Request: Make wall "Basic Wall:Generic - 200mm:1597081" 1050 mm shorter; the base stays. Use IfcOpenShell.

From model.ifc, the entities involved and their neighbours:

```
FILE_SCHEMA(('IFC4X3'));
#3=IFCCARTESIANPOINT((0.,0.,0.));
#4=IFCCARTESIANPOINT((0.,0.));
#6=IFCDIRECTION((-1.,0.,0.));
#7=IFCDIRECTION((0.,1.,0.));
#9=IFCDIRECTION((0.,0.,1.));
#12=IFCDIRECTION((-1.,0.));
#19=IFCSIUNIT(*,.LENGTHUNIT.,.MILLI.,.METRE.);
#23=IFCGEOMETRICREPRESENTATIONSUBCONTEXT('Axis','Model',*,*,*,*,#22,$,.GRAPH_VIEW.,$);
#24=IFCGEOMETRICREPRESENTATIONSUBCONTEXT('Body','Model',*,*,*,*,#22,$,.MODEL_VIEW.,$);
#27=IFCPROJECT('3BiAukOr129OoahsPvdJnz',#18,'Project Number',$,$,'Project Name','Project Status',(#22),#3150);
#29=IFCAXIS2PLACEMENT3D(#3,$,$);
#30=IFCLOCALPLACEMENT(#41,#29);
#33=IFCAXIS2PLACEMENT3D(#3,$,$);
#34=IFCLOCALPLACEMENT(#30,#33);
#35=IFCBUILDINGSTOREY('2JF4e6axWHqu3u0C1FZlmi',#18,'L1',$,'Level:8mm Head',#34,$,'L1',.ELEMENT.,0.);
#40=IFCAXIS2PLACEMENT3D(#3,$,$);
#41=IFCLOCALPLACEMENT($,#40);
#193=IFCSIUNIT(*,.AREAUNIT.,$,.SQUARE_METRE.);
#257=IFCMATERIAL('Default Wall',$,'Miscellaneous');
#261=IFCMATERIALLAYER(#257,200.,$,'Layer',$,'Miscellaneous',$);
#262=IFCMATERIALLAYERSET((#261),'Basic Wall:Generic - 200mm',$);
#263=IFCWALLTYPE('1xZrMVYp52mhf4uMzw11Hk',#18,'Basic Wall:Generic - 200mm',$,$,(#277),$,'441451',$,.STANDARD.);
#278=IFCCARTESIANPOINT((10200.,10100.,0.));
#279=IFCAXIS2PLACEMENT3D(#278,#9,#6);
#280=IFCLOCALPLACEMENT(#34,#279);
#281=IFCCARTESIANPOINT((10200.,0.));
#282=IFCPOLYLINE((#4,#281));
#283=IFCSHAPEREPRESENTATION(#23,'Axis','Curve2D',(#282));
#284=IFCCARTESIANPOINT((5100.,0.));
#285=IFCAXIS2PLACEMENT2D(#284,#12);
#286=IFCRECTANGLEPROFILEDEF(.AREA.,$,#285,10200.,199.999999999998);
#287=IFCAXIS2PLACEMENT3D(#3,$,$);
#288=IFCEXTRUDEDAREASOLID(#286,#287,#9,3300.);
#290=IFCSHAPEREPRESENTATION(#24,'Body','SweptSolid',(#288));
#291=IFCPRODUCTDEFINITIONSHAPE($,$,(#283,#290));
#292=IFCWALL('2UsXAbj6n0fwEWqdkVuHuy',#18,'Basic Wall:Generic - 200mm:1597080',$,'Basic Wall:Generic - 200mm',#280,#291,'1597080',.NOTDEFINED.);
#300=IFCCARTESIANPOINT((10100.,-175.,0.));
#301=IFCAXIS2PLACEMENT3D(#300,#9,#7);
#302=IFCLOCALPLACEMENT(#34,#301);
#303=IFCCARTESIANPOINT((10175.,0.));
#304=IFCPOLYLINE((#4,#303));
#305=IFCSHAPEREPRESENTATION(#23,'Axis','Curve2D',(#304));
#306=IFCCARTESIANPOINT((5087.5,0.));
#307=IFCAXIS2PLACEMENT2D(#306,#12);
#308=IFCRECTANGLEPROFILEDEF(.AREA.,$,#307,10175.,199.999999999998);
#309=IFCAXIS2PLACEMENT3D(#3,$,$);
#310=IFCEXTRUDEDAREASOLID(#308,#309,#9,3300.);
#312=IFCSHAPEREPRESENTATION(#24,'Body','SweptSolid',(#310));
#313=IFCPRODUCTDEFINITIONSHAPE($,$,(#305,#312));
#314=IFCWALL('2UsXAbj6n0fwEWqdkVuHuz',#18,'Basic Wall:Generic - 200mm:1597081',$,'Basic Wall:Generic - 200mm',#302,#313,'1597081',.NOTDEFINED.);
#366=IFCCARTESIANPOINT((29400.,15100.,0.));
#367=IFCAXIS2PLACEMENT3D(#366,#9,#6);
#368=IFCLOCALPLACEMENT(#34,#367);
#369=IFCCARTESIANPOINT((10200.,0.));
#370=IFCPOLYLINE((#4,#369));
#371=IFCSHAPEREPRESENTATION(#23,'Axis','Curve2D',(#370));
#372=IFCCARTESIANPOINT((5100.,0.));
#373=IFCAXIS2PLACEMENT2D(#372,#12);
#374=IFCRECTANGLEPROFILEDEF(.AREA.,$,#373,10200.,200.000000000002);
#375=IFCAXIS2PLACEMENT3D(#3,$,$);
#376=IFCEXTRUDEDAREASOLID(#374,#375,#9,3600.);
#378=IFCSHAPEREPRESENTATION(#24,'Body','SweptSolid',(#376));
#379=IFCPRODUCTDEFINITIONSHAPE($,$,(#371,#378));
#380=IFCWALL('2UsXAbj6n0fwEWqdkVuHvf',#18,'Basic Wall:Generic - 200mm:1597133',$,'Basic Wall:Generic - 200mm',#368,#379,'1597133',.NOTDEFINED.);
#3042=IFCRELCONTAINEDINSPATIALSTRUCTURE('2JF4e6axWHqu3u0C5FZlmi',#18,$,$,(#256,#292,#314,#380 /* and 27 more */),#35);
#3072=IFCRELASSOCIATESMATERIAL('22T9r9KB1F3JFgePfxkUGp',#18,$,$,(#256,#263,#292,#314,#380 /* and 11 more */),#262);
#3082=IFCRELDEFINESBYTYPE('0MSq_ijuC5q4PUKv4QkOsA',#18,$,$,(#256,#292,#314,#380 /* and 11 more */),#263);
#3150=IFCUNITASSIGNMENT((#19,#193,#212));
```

```python
import ifcopenshell
import ifcopenshell.geom
import ifcopenshell.util.representation
import ifcopenshell.util.shape
import ifcopenshell.util.unit

model = ifcopenshell.open("model.ifc")
unit_scale = ifcopenshell.util.unit.calculate_unit_scale(model)
settings = ifcopenshell.geom.settings()


def volume(element):
    """Net volume in cubic metres, openings subtracted."""
    shape = ifcopenshell.geom.create_shape(settings, element)
    return ifcopenshell.util.shape.get_volume(shape.geometry)


wall = model.by_id(314)
before = volume(wall)

body = ifcopenshell.util.representation.get_representation(wall, "Model", "Body")
solid = body.Items[0]
old_height = solid.Depth
solid.Depth -= 1.05 / unit_scale
after = volume(wall)

print(f"height {old_height:g} -> {solid.Depth:g}, volume {before:.3f} -> {after:.3f} m3")

model.write("model_edited.ifc")
```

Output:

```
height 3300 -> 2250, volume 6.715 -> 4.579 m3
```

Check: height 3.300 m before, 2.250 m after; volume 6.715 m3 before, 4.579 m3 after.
